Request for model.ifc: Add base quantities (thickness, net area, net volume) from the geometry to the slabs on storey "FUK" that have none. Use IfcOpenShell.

First a look at what the model holds.

```python
import ifcopenshell
import ifcopenshell.util.element
import ifcopenshell.util.unit

model = ifcopenshell.open("model.ifc")
print(model.schema)
for unit_type in ("LENGTHUNIT", "AREAUNIT", "VOLUMEUNIT"):
    print(unit_type, ifcopenshell.util.unit.calculate_unit_scale(model, unit_type))
storey = next(s for s in model.by_type("IfcBuildingStorey") if s.Name == "FUK")
slabs = [e for e in ifcopenshell.util.element.get_decomposition(storey) if e.is_a("IfcSlab")]
for e in sorted(slabs, key=lambda e: e.id()):
    print(e.id(), e.is_a(), e.Name, list(ifcopenshell.util.element.get_psets(e, qtos_only=True)), sep=" | ")
```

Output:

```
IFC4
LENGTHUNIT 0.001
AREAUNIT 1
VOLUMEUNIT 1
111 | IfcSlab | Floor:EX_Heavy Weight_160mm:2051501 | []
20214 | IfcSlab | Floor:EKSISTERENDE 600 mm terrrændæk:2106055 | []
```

```python
import ifcopenshell
import ifcopenshell.api.pset
import ifcopenshell.geom
import ifcopenshell.util.element
import ifcopenshell.util.shape
import ifcopenshell.util.unit

model = ifcopenshell.open("model.ifc")
unit_scale = ifcopenshell.util.unit.calculate_unit_scale(model)
area_scale = ifcopenshell.util.unit.calculate_unit_scale(model, "AREAUNIT")
volume_scale = ifcopenshell.util.unit.calculate_unit_scale(model, "VOLUMEUNIT")
settings = ifcopenshell.geom.settings()

storey = next(s for s in model.by_type("IfcBuildingStorey") if s.Name == "FUK")
slabs = [e for e in ifcopenshell.util.element.get_decomposition(storey) if e.is_a("IfcSlab")]

for e in sorted(slabs, key=lambda e: e.id()):
    if ifcopenshell.util.element.get_psets(e, qtos_only=True, should_inherit=False):
        continue
    # Geometry comes back in metres, in the element's own axes.
    shape = ifcopenshell.geom.create_shape(settings, e)
    values = {
        "Width": ifcopenshell.util.shape.get_z(shape.geometry) / unit_scale,
        "NetArea": ifcopenshell.util.shape.get_footprint_area(shape.geometry) / area_scale,
        "NetVolume": ifcopenshell.util.shape.get_volume(shape.geometry) / volume_scale,
    }
    qto = ifcopenshell.api.pset.add_qto(model, product=e, name="Qto_SlabBaseQuantities")
    ifcopenshell.api.pset.edit_qto(model, qto=qto, properties=values)
    print(e.id(), {k: round(v, 3) for k, v in values.items()})

model.write("model_edited.ifc")
```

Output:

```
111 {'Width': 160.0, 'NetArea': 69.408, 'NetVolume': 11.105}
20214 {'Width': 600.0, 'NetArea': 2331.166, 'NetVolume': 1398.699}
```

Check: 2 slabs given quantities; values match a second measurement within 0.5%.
